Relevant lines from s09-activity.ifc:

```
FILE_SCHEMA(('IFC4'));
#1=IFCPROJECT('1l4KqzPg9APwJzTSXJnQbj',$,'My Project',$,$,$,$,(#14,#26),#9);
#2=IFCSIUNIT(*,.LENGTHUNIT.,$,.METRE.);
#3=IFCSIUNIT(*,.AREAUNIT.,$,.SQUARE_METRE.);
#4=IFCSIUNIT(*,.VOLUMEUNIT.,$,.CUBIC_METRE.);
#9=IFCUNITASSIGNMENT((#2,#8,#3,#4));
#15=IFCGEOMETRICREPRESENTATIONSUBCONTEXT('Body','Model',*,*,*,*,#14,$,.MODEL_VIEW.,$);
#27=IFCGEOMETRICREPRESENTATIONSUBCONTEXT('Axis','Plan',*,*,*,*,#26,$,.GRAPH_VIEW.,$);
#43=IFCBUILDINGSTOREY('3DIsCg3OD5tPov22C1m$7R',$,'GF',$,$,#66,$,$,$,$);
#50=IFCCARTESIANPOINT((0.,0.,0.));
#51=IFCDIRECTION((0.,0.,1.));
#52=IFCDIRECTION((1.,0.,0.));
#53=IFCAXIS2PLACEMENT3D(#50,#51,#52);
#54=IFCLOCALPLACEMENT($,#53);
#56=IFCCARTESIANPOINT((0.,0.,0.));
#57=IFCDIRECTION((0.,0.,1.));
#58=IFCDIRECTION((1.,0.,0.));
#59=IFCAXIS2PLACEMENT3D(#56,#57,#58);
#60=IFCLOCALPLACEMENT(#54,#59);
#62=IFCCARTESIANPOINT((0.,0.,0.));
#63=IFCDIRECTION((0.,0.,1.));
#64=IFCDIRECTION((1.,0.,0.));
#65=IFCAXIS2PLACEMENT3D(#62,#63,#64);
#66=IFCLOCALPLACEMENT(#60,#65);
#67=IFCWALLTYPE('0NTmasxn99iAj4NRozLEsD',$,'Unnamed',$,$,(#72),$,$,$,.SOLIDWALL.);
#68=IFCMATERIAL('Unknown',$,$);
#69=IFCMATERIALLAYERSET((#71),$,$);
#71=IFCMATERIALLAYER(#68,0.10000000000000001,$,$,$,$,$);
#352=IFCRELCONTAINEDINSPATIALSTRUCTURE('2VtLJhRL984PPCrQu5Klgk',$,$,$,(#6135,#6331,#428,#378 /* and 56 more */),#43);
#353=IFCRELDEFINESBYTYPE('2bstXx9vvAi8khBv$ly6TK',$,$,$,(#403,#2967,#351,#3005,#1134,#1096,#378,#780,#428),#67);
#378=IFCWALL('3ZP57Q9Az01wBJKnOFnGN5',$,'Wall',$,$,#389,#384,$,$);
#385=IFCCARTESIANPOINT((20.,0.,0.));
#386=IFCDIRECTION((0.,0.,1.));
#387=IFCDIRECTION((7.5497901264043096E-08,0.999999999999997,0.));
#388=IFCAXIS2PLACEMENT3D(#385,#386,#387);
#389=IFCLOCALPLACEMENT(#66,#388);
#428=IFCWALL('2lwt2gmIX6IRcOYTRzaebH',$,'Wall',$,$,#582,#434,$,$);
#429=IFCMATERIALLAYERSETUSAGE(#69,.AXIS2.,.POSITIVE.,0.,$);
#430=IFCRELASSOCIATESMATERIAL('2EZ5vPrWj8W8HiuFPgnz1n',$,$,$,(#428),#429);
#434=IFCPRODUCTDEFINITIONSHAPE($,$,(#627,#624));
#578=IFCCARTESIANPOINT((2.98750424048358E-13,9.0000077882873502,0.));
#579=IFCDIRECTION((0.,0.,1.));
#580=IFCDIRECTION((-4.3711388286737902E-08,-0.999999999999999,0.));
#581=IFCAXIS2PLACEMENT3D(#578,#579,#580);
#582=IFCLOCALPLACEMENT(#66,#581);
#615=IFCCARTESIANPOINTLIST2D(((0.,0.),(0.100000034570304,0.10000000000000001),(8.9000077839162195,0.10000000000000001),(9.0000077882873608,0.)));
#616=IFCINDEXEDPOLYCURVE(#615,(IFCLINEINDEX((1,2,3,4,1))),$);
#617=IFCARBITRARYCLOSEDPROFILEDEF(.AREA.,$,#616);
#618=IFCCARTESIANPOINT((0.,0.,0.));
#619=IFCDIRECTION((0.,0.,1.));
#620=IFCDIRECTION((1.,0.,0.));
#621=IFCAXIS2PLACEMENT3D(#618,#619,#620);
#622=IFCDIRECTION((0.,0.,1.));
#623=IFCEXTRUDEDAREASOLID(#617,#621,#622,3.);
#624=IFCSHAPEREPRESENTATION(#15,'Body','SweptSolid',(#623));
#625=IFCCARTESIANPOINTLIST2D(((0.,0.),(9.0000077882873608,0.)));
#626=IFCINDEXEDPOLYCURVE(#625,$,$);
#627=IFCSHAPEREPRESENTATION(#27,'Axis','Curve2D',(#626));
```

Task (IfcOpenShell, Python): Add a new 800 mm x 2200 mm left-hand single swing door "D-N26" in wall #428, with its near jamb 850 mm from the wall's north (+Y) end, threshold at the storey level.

```python
import numpy as np
import ifcopenshell
import ifcopenshell.api.feature
import ifcopenshell.api.geometry
import ifcopenshell.api.root
import ifcopenshell.api.spatial
import ifcopenshell.geom
import ifcopenshell.util.element
import ifcopenshell.util.placement
import ifcopenshell.util.representation
import ifcopenshell.util.shape
import ifcopenshell.util.unit

model = ifcopenshell.open("s09-activity.ifc")
unit_scale = ifcopenshell.util.unit.calculate_unit_scale(model)
settings = ifcopenshell.geom.settings()


def volume(element):
    """Net volume in cubic metres, openings subtracted."""
    shape = ifcopenshell.geom.create_shape(settings, element)
    return ifcopenshell.util.shape.get_volume(shape.geometry)


wall = model.by_id(428)
storey = ifcopenshell.util.element.get_container(wall, ifc_class="IfcBuildingStorey")
context = ifcopenshell.util.representation.get_context(model, "Model", "Body", "MODEL_VIEW")
before = volume(wall)

width, height, from_end, sill = 0.8, 2.2, 0.85, 0.0  # metres

# The wall runs along its own X axis, and the end named is its -X end.
wall_shape = ifcopenshell.geom.create_shape(settings, wall)
x, y, z = ifcopenshell.util.shape.get_vertices(wall_shape.geometry).T
start = x.min() + from_end
face, thickness = float(y.min()), float(y.max() - y.min())
wall_matrix = ifcopenshell.util.placement.get_local_placement(wall.ObjectPlacement)
level = ifcopenshell.util.placement.get_local_placement(storey.ObjectPlacement)[2, 3]


def in_wall(x, y):
    """Placement at x, y metres in the wall's axes, at sill height."""
    matrix = wall_matrix.copy()
    matrix[:, 3] = wall_matrix @ np.array([x / unit_scale, y / unit_scale, 0.0, 1.0])
    matrix[2, 3] = level + sill / unit_scale
    return matrix


# Opening: a box that overshoots both wall faces by 50 mm.
opening = ifcopenshell.api.root.create_entity(model, ifc_class="IfcOpeningElement", predefined_type="OPENING")
box = ifcopenshell.api.geometry.add_wall_representation(
    model, context=context, length=width, height=height, thickness=thickness + 0.1
)
ifcopenshell.api.geometry.assign_representation(model, product=opening, representation=box)
ifcopenshell.api.geometry.edit_object_placement(model, product=opening, matrix=in_wall(start, face - 0.05), is_si=False)
ifcopenshell.api.feature.add_feature(model, feature=opening, element=wall)

door = ifcopenshell.api.root.create_entity(model, ifc_class="IfcDoor", name="D-N26", predefined_type="DOOR")
door.OverallWidth, door.OverallHeight = width / unit_scale, height / unit_scale
door.OperationType = "SINGLE_SWING_LEFT"
body = ifcopenshell.api.geometry.add_door_representation(
    model,
    context=context,
    overall_width=door.OverallWidth,
    overall_height=door.OverallHeight,
    operation_type="SINGLE_SWING_LEFT",
    lining_properties={"LiningDepth": thickness / unit_scale, "ThresholdDepth": thickness / unit_scale},
)
ifcopenshell.api.geometry.assign_representation(model, product=door, representation=body)
ifcopenshell.api.spatial.assign_container(model, products=[door], relating_structure=storey)
ifcopenshell.api.feature.add_filling(model, opening=opening, element=door)

# The lining spans the wall, so the door starts at the wall face.
ifcopenshell.api.geometry.edit_object_placement(model, product=door, matrix=in_wall(start, face), is_si=False)

after = volume(wall)

print(f"wall volume {before:.3f} -> {after:.3f} m3")

model.write("s09-activity-out.ifc")
```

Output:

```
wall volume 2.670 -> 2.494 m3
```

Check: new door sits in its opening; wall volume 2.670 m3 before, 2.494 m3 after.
